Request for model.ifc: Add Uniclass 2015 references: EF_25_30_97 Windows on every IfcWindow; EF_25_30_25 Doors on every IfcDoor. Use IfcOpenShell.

First a look at what the model holds.

```python
import ifcopenshell

model = ifcopenshell.open("model.ifc")
print(model.schema)
print("classifications:", [c.Name for c in model.by_type("IfcClassification")])
for ifc_class in ("IfcDoor", "IfcRoof", "IfcStair", "IfcWall", "IfcWindow"):
    print(ifc_class, len(model.by_type(ifc_class)))
```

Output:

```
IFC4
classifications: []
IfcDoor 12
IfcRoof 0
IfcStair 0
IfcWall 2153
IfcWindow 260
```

```python
import ifcopenshell
import ifcopenshell.api.classification

model = ifcopenshell.open("model.ifc")

system = ifcopenshell.api.classification.add_classification(model, classification="Uniclass 2015")

codes = {
    "IfcWindow": ("EF_25_30_97", "Windows"),
    "IfcDoor": ("EF_25_30_25", "Doors"),
}
for ifc_class, (code, name) in codes.items():
    products = model.by_type(ifc_class)
    ifcopenshell.api.classification.add_reference(
        model, products=products, classification=system, identification=code, name=name
    )
    print(code, len(products))

model.write("model_v2.ifc")
```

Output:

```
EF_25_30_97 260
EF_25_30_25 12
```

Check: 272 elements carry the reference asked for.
